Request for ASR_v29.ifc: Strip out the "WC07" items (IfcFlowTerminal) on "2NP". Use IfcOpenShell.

First a look at what the model holds.

```python
import ifcopenshell
import ifcopenshell.util.element

model = ifcopenshell.open("ASR_v29.ifc")
print(model.schema)
storey = next(s for s in model.by_type("IfcBuildingStorey") if s.Name == "2NP")
terminals = [e for e in ifcopenshell.util.element.get_decomposition(storey) if e.is_a("IfcFlowTerminal")]
seen = {}
for e in terminals:
    element_type = ifcopenshell.util.element.get_type(e)
    name = element_type.Name if element_type not in (None, e) else None
    seen[name] = seen.get(name, 0) + 1
for name, count in sorted(seen.items(), key=str):
    print(count, "x", name)
```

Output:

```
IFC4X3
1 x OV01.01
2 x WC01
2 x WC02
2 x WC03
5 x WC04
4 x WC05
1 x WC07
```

```python
import ifcopenshell
import ifcopenshell.api.root
import ifcopenshell.util.element

model = ifcopenshell.open("ASR_v29.ifc")

storey = next(s for s in model.by_type("IfcBuildingStorey") if s.Name == "2NP")
terminals = [e for e in ifcopenshell.util.element.get_decomposition(storey) if e.is_a("IfcFlowTerminal")]
targets = [e for e in terminals if (t := ifcopenshell.util.element.get_type(e)) not in (None, e) and t.Name == "WC07"]

for e in targets:
    ifcopenshell.api.root.remove_product(model, product=e)
print(len(targets), "removed")

model.write("ASR_v29_edited.ifc")
```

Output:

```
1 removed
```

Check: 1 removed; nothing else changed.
